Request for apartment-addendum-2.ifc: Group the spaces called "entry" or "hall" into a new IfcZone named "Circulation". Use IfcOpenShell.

First a look at what the model holds.

```python
import ifcopenshell

model = ifcopenshell.open("apartment-addendum-2.ifc")
print(model.schema)
seen = {}
for space in model.by_type("IfcSpace"):
    seen[space.LongName] = seen.get(space.LongName, 0) + 1
for name, count in sorted(seen.items(), key=str):
    print(count, "x", name)
print("zones:", [z.Name for z in model.by_type("IfcZone")][:20])
```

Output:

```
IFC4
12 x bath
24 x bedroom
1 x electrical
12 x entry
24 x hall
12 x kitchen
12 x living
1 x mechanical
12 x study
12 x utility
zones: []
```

```python
import ifcopenshell
import ifcopenshell.api.group
import ifcopenshell.api.root

model = ifcopenshell.open("apartment-addendum-2.ifc")

names = {"entry", "hall"}
spaces = [s for s in model.by_type("IfcSpace") if s.LongName in names]

zone = ifcopenshell.api.root.create_entity(model, ifc_class="IfcZone", name="Circulation")
ifcopenshell.api.group.assign_group(model, products=spaces, group=zone)
print(len(spaces), "spaces in", zone.Name)

model.write("apartment-addendum-2_updated.ifc")
```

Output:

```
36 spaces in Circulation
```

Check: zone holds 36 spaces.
